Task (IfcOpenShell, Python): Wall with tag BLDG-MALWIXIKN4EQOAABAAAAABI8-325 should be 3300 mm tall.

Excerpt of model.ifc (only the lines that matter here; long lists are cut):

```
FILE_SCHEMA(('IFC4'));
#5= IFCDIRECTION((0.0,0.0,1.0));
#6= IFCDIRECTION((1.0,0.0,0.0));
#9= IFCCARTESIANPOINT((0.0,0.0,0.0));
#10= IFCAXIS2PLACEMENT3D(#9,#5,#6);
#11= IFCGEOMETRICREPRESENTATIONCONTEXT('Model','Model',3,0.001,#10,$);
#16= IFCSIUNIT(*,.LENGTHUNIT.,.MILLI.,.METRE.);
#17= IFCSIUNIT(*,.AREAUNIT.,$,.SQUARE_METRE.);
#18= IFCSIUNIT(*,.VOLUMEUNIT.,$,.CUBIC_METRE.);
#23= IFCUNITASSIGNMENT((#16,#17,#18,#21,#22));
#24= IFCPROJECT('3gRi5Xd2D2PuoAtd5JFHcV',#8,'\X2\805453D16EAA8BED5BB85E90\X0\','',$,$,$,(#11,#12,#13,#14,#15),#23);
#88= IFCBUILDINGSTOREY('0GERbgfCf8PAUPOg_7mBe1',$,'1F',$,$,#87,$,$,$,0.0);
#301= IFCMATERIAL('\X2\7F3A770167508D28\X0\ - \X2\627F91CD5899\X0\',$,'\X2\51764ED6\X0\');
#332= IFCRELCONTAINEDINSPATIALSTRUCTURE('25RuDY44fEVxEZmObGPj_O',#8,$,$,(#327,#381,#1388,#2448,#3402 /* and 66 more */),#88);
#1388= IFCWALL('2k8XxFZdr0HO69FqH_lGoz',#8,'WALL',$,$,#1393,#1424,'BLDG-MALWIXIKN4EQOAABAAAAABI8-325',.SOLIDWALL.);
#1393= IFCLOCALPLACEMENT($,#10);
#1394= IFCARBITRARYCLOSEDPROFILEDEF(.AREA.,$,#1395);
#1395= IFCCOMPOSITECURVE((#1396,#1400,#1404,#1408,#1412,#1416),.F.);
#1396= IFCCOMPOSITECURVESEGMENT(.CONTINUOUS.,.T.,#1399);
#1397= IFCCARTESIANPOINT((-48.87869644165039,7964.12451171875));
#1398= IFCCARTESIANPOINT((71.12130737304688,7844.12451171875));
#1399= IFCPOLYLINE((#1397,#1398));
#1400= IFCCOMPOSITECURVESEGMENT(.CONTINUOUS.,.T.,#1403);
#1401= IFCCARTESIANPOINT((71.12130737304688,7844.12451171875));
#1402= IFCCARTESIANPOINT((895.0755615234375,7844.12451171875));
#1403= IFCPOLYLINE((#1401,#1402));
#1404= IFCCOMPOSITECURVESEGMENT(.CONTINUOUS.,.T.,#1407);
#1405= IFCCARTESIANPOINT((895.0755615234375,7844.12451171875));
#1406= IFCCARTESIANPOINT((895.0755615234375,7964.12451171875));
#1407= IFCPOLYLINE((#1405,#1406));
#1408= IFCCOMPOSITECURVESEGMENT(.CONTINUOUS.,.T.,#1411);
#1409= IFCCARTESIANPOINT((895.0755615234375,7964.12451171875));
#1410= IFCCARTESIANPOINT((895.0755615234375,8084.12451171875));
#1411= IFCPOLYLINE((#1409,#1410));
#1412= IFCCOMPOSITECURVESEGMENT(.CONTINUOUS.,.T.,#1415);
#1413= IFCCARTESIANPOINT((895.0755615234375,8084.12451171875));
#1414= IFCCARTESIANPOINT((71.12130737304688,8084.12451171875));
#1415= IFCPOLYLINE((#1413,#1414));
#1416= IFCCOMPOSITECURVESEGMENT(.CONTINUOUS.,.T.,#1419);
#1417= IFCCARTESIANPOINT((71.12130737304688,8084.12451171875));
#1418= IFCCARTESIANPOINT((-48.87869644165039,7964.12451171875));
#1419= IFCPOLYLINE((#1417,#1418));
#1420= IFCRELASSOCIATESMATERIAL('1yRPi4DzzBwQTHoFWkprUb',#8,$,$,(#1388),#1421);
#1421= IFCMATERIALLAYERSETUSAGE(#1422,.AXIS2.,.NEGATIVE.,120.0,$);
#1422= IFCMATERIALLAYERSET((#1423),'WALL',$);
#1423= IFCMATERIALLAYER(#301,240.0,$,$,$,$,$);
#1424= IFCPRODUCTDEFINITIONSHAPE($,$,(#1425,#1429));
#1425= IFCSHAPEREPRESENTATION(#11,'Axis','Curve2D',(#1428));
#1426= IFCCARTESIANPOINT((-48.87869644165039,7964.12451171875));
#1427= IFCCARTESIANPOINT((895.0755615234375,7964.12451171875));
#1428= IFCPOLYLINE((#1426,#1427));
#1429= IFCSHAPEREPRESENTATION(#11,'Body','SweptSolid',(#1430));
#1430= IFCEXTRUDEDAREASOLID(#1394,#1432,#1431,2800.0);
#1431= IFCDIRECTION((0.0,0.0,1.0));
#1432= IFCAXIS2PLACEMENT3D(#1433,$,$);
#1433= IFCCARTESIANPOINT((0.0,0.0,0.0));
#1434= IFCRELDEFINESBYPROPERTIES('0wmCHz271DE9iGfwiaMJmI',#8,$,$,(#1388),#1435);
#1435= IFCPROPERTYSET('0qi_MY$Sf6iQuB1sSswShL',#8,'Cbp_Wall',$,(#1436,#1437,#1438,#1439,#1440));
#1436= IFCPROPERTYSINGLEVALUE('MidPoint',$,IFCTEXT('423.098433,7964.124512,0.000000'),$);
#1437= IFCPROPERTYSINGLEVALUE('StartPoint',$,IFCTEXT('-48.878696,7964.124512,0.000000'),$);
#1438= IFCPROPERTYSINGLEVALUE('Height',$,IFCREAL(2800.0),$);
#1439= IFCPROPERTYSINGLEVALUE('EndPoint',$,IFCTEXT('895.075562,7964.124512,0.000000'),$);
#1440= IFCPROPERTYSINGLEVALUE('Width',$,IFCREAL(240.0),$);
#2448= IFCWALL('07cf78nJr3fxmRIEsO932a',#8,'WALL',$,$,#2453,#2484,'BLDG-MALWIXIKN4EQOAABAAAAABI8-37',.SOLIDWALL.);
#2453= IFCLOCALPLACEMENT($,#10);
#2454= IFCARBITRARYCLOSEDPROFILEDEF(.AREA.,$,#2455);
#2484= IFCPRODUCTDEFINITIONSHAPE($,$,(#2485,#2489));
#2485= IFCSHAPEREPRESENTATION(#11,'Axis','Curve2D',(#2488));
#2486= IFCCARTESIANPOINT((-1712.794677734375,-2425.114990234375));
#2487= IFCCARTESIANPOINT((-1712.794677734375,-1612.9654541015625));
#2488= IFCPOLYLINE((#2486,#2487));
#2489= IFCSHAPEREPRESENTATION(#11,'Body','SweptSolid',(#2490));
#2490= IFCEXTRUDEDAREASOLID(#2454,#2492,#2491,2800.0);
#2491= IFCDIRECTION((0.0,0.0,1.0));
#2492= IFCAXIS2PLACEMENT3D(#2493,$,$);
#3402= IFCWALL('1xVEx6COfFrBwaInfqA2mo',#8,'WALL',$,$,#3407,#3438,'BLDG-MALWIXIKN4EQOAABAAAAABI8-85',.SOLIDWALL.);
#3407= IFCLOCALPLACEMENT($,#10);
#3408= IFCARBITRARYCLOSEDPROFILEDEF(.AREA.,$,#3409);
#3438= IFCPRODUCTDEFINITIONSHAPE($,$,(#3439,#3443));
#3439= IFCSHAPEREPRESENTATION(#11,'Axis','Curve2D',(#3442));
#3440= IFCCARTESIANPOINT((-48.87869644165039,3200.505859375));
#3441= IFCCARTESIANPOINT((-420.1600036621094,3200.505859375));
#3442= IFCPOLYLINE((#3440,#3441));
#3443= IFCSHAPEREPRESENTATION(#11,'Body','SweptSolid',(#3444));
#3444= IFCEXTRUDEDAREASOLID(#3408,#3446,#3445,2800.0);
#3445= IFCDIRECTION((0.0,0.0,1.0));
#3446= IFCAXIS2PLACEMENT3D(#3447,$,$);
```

```python
import ifcopenshell
import ifcopenshell.api.pset
import ifcopenshell.geom
import ifcopenshell.util.element
import ifcopenshell.util.shape

model = ifcopenshell.open("model.ifc")
settings = ifcopenshell.geom.settings()


def volume(element):
    """Net volume in cubic metres, openings subtracted."""
    shape = ifcopenshell.geom.create_shape(settings, element)
    return ifcopenshell.util.shape.get_volume(shape.geometry)


wall = model.by_guid("2k8XxFZdr0HO69FqH_lGoz")
before = volume(wall)

body = next(r for r in wall.Representation.Representations if r.RepresentationIdentifier == "Body")
solid = body.Items[0]
old_height = solid.Depth
solid.Depth = 3300.0
after = volume(wall)

# Update the stored height, areas and volumes.
pset = model.by_id(ifcopenshell.util.element.get_pset(wall, "Cbp_Wall", should_inherit=False)["id"])
ifcopenshell.api.pset.edit_pset(model, pset=pset, properties={"Height": model.create_entity("IfcReal", solid.Depth)})

print(f"height {old_height:g} -> {solid.Depth:g}, volume {before:.3f} -> {after:.3f} m3")

model.write("model_rev.ifc")
```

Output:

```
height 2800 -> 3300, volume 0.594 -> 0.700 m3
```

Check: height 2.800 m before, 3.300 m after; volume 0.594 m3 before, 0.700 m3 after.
